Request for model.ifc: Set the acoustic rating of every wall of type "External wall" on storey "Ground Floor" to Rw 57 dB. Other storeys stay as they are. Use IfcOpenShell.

First a look at what the model holds.

```python
import ifcopenshell
import ifcopenshell.util.element

model = ifcopenshell.open("model.ifc")
print(model.schema)
storey = next(s for s in model.by_type("IfcBuildingStorey") if s.Name == "Ground Floor")
walls = [e for e in ifcopenshell.util.element.get_decomposition(storey) if e.is_a("IfcWall")]
seen = {}
for e in walls:
    element_type = ifcopenshell.util.element.get_type(e)
    key = (element_type.Name if element_type != e and element_type else None, ifcopenshell.util.element.get_pset(e, "Pset_WallCommon", "AcousticRating"))
    seen[key] = seen.get(key, 0) + 1
for (name, value), count in sorted(seen.items(), key=str):
    print(count, "x", name, "|", value)
```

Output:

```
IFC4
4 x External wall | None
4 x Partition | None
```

```python
import ifcopenshell
import ifcopenshell.api.pset
import ifcopenshell.util.element

model = ifcopenshell.open("model.ifc")

storey = next(s for s in model.by_type("IfcBuildingStorey") if s.Name == "Ground Floor")
walls = [e for e in ifcopenshell.util.element.get_decomposition(storey) if e.is_a("IfcWall")]

count = 0
for e in walls:
    element_type = ifcopenshell.util.element.get_type(e)
    if element_type in (None, e) or element_type.Name != "External wall":
        continue
    # add_pset returns the element's existing set when there is one.
    pset = ifcopenshell.api.pset.add_pset(model, product=e, name="Pset_WallCommon")
    ifcopenshell.api.pset.edit_pset(model, pset=pset, properties={"AcousticRating": "Rw 57 dB"})
    count += 1

print(count, "walls updated")

model.write("model_edited.ifc")
```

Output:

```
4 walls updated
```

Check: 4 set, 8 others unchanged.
